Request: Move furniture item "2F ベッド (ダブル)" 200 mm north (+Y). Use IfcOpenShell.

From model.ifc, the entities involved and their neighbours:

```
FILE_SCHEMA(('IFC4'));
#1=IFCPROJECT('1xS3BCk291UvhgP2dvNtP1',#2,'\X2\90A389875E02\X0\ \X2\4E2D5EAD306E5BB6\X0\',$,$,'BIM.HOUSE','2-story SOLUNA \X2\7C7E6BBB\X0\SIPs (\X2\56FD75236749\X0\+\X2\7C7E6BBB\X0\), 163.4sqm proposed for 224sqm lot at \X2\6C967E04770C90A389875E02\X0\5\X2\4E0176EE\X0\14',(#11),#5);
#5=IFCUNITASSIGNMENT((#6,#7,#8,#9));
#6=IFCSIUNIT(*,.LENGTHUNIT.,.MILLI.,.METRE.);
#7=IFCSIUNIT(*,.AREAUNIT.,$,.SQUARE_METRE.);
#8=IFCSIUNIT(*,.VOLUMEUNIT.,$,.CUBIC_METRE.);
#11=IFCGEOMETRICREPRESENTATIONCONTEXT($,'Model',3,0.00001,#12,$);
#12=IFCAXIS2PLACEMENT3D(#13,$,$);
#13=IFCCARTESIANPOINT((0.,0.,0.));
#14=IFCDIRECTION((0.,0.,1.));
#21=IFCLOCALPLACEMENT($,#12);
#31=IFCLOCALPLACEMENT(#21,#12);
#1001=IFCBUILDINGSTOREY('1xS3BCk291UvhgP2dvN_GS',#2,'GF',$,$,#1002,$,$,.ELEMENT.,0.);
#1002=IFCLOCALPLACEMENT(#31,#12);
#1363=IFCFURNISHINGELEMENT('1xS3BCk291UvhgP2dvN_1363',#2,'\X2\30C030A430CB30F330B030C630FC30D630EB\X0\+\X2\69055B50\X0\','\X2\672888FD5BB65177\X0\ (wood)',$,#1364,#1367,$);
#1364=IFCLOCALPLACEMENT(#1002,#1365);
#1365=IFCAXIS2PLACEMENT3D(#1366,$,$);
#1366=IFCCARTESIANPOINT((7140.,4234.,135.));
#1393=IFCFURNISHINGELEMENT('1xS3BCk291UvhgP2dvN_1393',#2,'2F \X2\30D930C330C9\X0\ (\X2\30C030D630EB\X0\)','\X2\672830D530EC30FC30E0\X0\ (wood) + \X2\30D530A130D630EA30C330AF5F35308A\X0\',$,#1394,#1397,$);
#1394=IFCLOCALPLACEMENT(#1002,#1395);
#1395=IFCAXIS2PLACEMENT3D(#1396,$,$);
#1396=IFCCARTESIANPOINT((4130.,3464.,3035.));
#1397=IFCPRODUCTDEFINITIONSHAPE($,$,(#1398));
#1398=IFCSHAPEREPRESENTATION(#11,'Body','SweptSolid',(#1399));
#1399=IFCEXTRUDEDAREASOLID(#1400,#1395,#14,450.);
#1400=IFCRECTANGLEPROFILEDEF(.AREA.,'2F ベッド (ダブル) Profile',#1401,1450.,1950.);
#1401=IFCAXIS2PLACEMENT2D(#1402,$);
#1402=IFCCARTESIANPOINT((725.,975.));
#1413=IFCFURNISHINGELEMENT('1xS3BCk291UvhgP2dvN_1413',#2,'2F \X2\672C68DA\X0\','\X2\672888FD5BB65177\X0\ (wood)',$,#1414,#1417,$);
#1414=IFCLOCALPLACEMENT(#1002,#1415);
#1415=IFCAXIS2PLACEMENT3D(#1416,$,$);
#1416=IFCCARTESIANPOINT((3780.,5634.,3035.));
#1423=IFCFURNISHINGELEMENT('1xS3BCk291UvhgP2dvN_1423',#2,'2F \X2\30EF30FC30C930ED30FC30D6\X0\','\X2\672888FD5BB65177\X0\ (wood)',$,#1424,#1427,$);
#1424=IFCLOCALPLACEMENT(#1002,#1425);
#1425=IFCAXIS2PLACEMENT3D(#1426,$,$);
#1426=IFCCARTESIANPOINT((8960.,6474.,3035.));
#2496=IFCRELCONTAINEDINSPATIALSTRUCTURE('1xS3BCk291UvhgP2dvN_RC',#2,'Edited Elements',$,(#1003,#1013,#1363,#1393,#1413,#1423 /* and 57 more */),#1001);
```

```python
import ifcopenshell
import ifcopenshell.api.geometry
import ifcopenshell.util.placement

model = ifcopenshell.open("model.ifc")

item = model.by_guid("1xS3BCk291UvhgP2dvN_1393")
matrix = ifcopenshell.util.placement.get_local_placement(item.ObjectPlacement)
matrix[1, 3] += 200.0
ifcopenshell.api.geometry.edit_object_placement(model, product=item, matrix=matrix, is_si=False)

print(ifcopenshell.util.placement.get_local_placement(item.ObjectPlacement).round(3) + 0.0)

model.write("model_v2.ifc")
```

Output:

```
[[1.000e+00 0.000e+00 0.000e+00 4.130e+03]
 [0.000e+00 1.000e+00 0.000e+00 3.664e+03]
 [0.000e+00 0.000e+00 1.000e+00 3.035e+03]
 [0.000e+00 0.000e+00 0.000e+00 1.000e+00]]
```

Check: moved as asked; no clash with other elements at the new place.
